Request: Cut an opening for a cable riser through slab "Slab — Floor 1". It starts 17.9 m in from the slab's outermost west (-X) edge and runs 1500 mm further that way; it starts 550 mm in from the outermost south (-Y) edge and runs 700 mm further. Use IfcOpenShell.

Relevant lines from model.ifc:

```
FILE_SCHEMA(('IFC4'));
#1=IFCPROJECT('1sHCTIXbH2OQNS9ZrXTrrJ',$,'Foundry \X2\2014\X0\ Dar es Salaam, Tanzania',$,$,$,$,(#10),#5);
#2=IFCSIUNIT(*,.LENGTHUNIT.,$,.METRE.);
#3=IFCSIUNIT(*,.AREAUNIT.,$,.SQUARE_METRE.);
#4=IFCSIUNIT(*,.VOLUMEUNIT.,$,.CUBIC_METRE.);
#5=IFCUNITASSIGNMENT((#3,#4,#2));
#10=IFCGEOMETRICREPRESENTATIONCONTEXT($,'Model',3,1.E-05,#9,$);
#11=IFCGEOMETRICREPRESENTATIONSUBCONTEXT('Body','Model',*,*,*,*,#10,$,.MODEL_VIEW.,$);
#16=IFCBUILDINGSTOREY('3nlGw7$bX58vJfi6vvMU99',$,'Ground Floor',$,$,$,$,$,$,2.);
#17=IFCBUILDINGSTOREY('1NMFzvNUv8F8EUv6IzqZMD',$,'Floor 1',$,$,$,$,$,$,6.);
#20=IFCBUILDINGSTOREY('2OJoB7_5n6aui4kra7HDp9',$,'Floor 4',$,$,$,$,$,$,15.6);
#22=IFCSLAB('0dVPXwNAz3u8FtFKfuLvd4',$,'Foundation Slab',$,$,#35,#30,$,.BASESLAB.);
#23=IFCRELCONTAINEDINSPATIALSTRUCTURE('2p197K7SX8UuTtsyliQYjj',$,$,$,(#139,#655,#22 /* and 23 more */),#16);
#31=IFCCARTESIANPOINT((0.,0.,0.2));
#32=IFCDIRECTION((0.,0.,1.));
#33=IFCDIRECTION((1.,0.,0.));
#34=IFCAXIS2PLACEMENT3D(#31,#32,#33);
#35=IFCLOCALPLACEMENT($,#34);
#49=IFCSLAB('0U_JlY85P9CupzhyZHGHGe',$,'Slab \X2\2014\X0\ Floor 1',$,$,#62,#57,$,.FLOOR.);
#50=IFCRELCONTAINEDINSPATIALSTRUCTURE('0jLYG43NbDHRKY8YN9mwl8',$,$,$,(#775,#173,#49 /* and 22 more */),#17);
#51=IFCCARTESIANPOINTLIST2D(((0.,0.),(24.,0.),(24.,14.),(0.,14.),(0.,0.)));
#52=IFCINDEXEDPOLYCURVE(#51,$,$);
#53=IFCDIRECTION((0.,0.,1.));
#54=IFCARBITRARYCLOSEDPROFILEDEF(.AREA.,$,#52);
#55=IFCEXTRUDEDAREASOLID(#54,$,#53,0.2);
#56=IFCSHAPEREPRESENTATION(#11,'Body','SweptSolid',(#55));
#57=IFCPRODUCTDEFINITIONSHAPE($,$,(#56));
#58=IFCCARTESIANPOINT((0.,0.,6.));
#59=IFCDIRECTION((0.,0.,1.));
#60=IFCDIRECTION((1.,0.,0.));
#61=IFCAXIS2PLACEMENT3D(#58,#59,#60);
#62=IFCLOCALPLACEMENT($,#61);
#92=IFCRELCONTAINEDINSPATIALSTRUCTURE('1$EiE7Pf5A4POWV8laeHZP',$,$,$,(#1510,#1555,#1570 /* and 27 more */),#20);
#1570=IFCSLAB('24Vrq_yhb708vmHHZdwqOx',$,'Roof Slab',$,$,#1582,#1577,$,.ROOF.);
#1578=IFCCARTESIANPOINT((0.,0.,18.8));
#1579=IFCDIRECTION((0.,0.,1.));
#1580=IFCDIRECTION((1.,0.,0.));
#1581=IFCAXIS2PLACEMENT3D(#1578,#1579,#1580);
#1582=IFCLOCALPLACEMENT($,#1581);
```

```python
import numpy as np
import ifcopenshell
import ifcopenshell.api.feature
import ifcopenshell.api.geometry
import ifcopenshell.api.root
import ifcopenshell.geom
import ifcopenshell.util.placement
import ifcopenshell.util.representation
import ifcopenshell.util.shape
import ifcopenshell.util.unit

model = ifcopenshell.open("model.ifc")
unit_scale = ifcopenshell.util.unit.calculate_unit_scale(model)
settings = ifcopenshell.geom.settings()


def volume(element):
    """Net volume in cubic metres, openings subtracted."""
    shape = ifcopenshell.geom.create_shape(settings, element)
    return ifcopenshell.util.shape.get_volume(shape.geometry)


slab = model.by_guid("0U_JlY85P9CupzhyZHGHGe")
before = volume(slab)

# Extent in the slab's own axes, in metres. The edges named are its -X and -Y sides.
slab_shape = ifcopenshell.geom.create_shape(settings, slab)
vertices = ifcopenshell.util.shape.get_vertices(slab_shape.geometry)
x_min, y_min, bottom = vertices.min(axis=0)
top = vertices[:, 2].max()

opening = ifcopenshell.api.root.create_entity(model, ifc_class="IfcOpeningElement", name="Cable riser opening", predefined_type="OPENING")
context = ifcopenshell.util.representation.get_context(model, "Model", "Body", "MODEL_VIEW")
width, depth = 1.5, 0.7
outline = [(0.0, 0.0), (width, 0.0), (width, depth), (0.0, depth), (0.0, 0.0)]
# Overshoot both faces by 50 mm so the cut is clean.
shape = ifcopenshell.api.geometry.add_slab_representation(
    model, context=context, depth=top - bottom + 0.1, polyline=outline
)
ifcopenshell.api.geometry.assign_representation(model, product=opening, representation=shape)

matrix = ifcopenshell.util.placement.get_local_placement(slab.ObjectPlacement)
matrix[:, 3] = matrix @ np.append(np.array([x_min + 17.9, y_min + 0.55, bottom - 0.05]) / unit_scale, 1.0)
ifcopenshell.api.geometry.edit_object_placement(model, product=opening, matrix=matrix, is_si=False)
ifcopenshell.api.feature.add_feature(model, feature=opening, element=slab)

after = volume(slab)

print(f"slab volume {before:.3f} -> {after:.3f} m3")

model.write("model_edited.ifc")
```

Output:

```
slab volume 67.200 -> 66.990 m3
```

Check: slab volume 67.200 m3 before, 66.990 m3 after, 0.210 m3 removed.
